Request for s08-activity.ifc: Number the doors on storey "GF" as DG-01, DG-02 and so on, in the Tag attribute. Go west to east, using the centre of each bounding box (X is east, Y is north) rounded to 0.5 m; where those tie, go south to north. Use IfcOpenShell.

First a look at what the model holds.

```python
import ifcopenshell
import ifcopenshell.util.element
import ifcopenshell.util.placement

model = ifcopenshell.open("s08-activity.ifc")
print(model.schema)
storey = next(s for s in model.by_type("IfcBuildingStorey") if s.Name == "GF")
doors = [e for e in ifcopenshell.util.element.get_decomposition(storey) if e.is_a("IfcDoor")]
for e in sorted(doors, key=lambda e: e.id()):
    origin = ifcopenshell.util.placement.get_local_placement(e.ObjectPlacement)[:3, 3]
    print(e.id(), e.Tag, e.Name, origin.round(2) + 0.0, sep=" | ")
```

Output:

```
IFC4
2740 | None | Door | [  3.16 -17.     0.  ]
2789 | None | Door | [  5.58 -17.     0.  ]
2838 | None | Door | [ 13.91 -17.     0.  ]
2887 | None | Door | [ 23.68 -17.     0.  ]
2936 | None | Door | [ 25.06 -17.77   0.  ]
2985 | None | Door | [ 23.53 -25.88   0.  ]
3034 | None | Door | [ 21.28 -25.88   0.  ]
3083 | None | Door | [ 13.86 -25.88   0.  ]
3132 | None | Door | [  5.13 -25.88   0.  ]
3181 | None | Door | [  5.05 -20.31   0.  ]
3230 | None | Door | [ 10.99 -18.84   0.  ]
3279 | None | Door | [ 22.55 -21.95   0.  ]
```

```python
import ifcopenshell
import ifcopenshell.geom
import ifcopenshell.util.element
import ifcopenshell.util.shape

model = ifcopenshell.open("s08-activity.ifc")
settings = ifcopenshell.geom.settings()
settings.set("use-world-coords", True)


def centre(element):
    shape = ifcopenshell.geom.create_shape(settings, element)
    return ifcopenshell.util.shape.get_bbox_centroid(shape.geometry)


storey = next(s for s in model.by_type("IfcBuildingStorey") if s.Name == "GF")
doors = [e for e in ifcopenshell.util.element.get_decomposition(storey) if e.is_a("IfcDoor")]

# Insertion points can sit at a corner or the storey origin, so sort by the geometry (in metres).
centres = {e: centre(e) for e in doors}
doors.sort(key=lambda e: (round(centres[e][0] / 0.5), centres[e][1]))

for i, e in enumerate(doors, start=1):
    number = f"DG-{i:02d}"
    e.Tag = number
    print(e.id(), number)

model.write("s08-activity_updated.ifc")
```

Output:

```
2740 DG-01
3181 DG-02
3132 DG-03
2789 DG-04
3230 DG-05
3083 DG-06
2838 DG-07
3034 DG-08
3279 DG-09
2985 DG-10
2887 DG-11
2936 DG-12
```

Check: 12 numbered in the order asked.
